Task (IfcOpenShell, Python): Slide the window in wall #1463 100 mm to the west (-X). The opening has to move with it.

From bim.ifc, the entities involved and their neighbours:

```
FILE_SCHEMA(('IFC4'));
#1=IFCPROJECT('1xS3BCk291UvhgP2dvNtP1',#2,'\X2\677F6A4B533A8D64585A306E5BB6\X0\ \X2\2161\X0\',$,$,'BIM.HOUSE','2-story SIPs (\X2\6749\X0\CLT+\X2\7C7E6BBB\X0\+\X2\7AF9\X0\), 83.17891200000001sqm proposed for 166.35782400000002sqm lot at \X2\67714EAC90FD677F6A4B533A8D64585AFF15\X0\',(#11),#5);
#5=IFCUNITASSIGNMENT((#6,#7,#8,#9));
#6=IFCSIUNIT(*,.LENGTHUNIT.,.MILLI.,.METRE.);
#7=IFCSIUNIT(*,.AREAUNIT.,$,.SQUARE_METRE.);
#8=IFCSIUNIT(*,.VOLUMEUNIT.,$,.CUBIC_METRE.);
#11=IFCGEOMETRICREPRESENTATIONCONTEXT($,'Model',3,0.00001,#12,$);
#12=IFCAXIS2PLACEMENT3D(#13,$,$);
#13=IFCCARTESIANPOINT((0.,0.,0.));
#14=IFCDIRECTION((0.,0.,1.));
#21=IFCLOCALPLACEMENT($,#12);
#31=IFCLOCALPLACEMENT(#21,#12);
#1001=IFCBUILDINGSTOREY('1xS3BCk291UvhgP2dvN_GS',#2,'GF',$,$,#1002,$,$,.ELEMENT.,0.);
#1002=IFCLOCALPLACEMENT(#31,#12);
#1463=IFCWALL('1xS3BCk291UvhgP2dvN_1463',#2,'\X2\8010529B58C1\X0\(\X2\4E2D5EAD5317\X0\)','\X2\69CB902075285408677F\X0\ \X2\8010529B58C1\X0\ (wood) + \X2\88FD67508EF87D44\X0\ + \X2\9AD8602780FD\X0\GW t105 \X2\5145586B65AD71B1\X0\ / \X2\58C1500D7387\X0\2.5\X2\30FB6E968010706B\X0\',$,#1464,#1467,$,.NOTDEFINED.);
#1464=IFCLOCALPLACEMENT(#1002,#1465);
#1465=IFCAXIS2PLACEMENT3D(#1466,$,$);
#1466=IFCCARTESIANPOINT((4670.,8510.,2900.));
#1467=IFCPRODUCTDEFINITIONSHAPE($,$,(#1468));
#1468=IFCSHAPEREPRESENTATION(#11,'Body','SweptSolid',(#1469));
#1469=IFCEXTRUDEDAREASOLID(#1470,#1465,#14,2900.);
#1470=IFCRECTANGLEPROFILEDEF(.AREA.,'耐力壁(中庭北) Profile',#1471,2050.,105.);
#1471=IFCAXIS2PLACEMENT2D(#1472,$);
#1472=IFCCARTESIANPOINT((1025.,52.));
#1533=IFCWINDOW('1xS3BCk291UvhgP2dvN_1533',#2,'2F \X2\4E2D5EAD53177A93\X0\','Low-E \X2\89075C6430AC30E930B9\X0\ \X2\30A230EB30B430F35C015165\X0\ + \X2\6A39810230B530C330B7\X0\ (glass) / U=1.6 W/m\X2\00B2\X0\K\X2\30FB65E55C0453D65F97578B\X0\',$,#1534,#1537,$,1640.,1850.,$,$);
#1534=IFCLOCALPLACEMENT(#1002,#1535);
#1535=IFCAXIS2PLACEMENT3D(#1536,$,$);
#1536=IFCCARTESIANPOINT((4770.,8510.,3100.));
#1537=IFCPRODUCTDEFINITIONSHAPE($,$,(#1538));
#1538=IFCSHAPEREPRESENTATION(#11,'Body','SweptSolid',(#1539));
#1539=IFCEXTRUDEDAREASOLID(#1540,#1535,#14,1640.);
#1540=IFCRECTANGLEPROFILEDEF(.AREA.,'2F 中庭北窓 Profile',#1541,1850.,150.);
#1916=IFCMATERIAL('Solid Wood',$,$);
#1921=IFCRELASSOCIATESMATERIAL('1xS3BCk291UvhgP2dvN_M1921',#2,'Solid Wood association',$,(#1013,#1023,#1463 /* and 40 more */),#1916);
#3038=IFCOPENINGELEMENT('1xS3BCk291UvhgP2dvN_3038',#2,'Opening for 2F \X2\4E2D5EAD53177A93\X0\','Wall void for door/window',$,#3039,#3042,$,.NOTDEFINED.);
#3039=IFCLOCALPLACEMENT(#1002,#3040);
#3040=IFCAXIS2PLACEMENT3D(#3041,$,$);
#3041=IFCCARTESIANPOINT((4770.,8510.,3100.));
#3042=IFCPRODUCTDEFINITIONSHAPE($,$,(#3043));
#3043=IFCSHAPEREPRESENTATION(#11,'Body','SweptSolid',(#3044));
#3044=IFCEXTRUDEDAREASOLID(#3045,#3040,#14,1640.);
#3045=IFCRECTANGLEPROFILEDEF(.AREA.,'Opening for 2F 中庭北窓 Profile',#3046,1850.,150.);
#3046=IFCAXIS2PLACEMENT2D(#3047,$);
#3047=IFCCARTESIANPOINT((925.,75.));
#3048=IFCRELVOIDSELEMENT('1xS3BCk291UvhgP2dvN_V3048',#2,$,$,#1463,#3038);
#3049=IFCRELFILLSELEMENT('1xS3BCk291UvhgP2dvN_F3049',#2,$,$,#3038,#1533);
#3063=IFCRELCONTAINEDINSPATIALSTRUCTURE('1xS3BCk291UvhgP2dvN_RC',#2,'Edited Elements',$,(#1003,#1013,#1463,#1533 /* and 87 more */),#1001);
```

```python
import ifcopenshell
import ifcopenshell.api.geometry
import ifcopenshell.util.placement

model = ifcopenshell.open("bim.ifc")

window = model.by_guid("1xS3BCk291UvhgP2dvN_1533")
opening = window.FillsVoids[0].RelatingOpeningElement
wall = opening.VoidsElements[0].RelatingBuildingElement

wall_matrix = ifcopenshell.util.placement.get_local_placement(wall.ObjectPlacement)
shift = wall_matrix[:3, 0] * -100.0
before = ifcopenshell.util.placement.get_local_placement(window.ObjectPlacement)[:3, 3].copy()

# The window is not placed relative to its opening, so move both.
for product in (opening, window):
    matrix = ifcopenshell.util.placement.get_local_placement(product.ObjectPlacement)
    matrix[:3, 3] += shift
    ifcopenshell.api.geometry.edit_object_placement(model, product=product, matrix=matrix, is_si=False)

after = ifcopenshell.util.placement.get_local_placement(window.ObjectPlacement)[:3, 3]
print("window moved by", (after - before).round(3) + 0.0)

model.write("bim_rev.ifc")
```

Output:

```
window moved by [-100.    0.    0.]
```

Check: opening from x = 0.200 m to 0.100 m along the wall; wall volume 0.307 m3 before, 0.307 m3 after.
